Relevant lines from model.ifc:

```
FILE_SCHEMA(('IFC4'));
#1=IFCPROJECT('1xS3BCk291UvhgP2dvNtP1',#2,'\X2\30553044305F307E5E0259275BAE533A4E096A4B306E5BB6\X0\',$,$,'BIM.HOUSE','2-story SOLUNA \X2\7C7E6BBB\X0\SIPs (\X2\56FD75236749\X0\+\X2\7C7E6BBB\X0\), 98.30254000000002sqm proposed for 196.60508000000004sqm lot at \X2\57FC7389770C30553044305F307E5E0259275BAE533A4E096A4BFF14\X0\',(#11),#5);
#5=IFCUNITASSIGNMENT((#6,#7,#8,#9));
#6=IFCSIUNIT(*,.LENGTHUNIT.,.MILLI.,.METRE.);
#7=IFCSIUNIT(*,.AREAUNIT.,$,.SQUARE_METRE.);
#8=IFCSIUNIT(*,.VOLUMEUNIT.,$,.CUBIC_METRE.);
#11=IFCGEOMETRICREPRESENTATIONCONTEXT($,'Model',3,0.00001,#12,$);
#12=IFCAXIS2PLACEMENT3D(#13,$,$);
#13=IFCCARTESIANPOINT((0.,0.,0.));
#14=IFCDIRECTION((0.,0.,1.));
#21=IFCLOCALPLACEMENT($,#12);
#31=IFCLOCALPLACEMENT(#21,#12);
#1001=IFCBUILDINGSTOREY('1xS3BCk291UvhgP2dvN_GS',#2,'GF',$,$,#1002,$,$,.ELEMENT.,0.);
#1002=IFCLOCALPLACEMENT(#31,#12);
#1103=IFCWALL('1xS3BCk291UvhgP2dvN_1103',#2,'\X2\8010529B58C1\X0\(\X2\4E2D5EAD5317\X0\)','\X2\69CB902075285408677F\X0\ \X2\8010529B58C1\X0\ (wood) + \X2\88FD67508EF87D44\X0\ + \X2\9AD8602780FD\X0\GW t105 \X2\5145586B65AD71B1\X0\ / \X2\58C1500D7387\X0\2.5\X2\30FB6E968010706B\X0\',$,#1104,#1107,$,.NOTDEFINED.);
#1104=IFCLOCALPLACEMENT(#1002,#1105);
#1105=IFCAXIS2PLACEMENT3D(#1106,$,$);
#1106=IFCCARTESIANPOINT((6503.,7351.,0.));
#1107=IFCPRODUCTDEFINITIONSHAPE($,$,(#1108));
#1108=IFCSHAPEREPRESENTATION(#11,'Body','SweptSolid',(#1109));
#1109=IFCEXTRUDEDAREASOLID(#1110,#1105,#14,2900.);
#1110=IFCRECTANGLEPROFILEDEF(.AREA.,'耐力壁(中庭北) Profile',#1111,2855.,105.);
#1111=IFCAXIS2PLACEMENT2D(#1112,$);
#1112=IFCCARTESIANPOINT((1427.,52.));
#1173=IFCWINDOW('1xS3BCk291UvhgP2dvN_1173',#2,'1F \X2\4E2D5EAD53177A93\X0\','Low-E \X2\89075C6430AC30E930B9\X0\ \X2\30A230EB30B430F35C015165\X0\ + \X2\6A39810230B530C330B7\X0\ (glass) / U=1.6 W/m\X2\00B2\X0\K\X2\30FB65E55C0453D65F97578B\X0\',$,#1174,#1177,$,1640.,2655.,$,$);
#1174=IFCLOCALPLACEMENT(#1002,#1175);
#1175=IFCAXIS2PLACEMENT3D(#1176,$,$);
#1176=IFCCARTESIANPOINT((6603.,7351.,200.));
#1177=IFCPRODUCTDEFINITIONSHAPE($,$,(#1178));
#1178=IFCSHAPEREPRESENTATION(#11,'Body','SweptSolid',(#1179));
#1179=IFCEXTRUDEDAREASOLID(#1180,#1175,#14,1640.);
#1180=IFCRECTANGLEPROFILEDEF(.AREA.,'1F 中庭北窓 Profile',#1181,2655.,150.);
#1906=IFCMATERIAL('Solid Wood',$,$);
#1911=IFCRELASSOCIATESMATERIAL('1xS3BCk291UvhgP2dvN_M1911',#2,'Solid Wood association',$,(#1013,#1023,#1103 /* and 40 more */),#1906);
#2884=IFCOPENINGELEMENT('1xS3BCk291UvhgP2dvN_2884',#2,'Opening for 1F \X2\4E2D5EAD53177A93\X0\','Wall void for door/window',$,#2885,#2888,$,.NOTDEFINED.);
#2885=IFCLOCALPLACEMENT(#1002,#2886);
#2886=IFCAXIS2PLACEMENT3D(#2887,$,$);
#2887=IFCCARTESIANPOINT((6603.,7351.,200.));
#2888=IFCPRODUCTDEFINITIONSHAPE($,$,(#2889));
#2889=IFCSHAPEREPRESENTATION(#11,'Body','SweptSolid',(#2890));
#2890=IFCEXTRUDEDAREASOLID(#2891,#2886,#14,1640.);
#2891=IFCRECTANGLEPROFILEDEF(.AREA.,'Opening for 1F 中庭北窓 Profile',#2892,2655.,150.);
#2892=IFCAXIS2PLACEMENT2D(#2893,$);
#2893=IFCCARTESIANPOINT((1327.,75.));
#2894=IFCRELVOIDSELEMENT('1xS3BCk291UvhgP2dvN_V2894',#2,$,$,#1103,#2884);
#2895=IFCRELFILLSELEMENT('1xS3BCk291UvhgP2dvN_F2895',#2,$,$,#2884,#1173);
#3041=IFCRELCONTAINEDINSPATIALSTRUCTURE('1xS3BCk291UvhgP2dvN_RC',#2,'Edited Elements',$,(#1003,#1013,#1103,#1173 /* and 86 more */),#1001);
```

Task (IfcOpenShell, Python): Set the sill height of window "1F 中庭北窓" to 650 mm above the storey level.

```python
import numpy as np
import ifcopenshell
import ifcopenshell.api.geometry
import ifcopenshell.geom
import ifcopenshell.util.element
import ifcopenshell.util.placement
import ifcopenshell.util.shape
import ifcopenshell.util.unit

model = ifcopenshell.open("model.ifc")
unit_scale = ifcopenshell.util.unit.calculate_unit_scale(model)

window = model.by_guid("1xS3BCk291UvhgP2dvN_1173")
opening = window.FillsVoids[0].RelatingOpeningElement
storey = ifcopenshell.util.element.get_container(window, ifc_class="IfcBuildingStorey")
level = ifcopenshell.util.placement.get_local_placement(storey.ObjectPlacement)[2, 3]

# The opening's origin need not be at the sill, so measure its lowest point.
shape = ifcopenshell.geom.create_shape(ifcopenshell.geom.settings(), opening)
bottom = ifcopenshell.util.shape.get_shape_bottom_elevation(shape, shape.geometry) / unit_scale
dz = level + 650.0 - bottom

shift = np.array([0.0, 0.0, dz])
# The window is not placed relative to its opening, so move both.
for product in (opening, window):
    matrix = ifcopenshell.util.placement.get_local_placement(product.ObjectPlacement)
    matrix[:3, 3] += shift
    ifcopenshell.api.geometry.edit_object_placement(model, product=product, matrix=matrix, is_si=False)

print(f"moved by {dz * unit_scale:+.3f} m")

model.write("model_v2.ifc")
```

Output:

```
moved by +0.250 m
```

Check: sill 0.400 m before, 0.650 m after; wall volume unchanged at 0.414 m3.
